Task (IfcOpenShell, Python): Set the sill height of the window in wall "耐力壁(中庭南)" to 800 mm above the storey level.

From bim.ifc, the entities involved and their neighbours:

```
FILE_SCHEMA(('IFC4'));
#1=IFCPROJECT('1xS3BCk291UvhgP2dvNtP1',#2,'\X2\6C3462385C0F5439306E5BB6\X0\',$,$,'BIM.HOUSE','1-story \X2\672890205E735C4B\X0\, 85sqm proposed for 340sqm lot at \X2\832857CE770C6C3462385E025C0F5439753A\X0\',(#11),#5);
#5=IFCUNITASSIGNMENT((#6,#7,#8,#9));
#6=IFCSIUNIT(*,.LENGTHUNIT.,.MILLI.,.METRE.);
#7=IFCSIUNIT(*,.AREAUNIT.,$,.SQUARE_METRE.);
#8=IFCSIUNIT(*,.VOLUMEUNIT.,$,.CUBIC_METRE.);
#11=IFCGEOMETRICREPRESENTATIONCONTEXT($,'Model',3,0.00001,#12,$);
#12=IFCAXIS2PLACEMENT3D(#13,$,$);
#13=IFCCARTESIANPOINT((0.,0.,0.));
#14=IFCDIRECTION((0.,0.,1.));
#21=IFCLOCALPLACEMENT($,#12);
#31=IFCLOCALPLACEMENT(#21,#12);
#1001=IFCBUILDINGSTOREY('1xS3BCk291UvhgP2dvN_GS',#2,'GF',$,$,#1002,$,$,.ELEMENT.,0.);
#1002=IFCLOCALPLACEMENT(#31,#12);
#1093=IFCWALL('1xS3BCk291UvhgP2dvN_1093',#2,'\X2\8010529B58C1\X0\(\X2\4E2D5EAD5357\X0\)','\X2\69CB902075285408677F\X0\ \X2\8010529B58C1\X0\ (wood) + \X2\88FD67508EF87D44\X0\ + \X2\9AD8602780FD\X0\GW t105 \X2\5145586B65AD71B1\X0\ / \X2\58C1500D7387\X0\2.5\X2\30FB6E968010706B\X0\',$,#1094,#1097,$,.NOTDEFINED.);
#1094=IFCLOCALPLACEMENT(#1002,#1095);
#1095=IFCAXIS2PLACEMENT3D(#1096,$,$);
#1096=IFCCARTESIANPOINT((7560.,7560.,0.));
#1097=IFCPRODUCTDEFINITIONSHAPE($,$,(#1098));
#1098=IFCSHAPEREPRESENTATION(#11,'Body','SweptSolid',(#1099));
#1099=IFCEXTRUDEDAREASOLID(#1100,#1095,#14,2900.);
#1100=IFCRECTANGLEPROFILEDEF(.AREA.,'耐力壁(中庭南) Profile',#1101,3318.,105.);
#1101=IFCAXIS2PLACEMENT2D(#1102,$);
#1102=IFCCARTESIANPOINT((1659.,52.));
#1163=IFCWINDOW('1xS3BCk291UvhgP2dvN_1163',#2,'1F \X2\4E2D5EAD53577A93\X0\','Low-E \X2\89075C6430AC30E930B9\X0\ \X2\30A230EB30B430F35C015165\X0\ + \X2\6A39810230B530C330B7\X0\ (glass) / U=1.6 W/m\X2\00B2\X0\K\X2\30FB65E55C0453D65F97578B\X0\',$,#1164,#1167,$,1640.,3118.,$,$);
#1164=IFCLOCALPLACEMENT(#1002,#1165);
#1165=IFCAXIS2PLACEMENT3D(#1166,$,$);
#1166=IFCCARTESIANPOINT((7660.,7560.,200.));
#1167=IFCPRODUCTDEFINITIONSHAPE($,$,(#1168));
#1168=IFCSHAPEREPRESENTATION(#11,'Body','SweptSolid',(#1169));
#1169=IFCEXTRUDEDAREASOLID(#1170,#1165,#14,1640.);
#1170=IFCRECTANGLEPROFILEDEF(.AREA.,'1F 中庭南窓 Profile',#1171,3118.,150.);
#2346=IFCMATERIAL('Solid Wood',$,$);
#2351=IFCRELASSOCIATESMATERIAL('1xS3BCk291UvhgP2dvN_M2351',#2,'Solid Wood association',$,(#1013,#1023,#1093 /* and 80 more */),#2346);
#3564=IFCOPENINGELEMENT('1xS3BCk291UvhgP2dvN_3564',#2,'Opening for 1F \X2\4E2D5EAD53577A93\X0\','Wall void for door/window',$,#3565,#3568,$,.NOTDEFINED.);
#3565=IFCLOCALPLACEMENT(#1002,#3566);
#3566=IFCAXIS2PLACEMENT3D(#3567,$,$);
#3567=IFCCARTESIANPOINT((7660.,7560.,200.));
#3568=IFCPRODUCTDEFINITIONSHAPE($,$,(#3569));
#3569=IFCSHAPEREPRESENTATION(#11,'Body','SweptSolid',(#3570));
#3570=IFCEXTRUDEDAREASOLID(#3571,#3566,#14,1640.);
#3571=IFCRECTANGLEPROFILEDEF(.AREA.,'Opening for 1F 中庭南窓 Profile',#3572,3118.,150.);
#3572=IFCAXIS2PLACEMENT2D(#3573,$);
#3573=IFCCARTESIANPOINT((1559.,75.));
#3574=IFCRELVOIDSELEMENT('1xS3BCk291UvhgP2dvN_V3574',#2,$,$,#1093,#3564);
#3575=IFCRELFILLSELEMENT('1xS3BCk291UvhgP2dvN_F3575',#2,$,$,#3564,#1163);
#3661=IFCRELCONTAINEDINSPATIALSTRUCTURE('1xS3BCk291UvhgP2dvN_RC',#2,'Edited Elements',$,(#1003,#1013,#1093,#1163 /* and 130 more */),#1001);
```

```python
import numpy as np
import ifcopenshell
import ifcopenshell.api.geometry
import ifcopenshell.geom
import ifcopenshell.util.element
import ifcopenshell.util.placement
import ifcopenshell.util.shape
import ifcopenshell.util.unit

model = ifcopenshell.open("bim.ifc")
unit_scale = ifcopenshell.util.unit.calculate_unit_scale(model)

window = model.by_guid("1xS3BCk291UvhgP2dvN_1163")
opening = window.FillsVoids[0].RelatingOpeningElement
storey = ifcopenshell.util.element.get_container(window, ifc_class="IfcBuildingStorey")
level = ifcopenshell.util.placement.get_local_placement(storey.ObjectPlacement)[2, 3]

# The opening's origin need not be at the sill, so measure its lowest point.
shape = ifcopenshell.geom.create_shape(ifcopenshell.geom.settings(), opening)
bottom = ifcopenshell.util.shape.get_shape_bottom_elevation(shape, shape.geometry) / unit_scale
dz = level + 0.8 / unit_scale - bottom

shift = np.array([0.0, 0.0, dz])
# The window is not placed relative to its opening, so move both.
for product in (opening, window):
    matrix = ifcopenshell.util.placement.get_local_placement(product.ObjectPlacement)
    matrix[:3, 3] += shift
    ifcopenshell.api.geometry.edit_object_placement(model, product=product, matrix=matrix, is_si=False)

print(f"moved by {dz * unit_scale:+.3f} m")

model.write("bim_edited.ifc")
```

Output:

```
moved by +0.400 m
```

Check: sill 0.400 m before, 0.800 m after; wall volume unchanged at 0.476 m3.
